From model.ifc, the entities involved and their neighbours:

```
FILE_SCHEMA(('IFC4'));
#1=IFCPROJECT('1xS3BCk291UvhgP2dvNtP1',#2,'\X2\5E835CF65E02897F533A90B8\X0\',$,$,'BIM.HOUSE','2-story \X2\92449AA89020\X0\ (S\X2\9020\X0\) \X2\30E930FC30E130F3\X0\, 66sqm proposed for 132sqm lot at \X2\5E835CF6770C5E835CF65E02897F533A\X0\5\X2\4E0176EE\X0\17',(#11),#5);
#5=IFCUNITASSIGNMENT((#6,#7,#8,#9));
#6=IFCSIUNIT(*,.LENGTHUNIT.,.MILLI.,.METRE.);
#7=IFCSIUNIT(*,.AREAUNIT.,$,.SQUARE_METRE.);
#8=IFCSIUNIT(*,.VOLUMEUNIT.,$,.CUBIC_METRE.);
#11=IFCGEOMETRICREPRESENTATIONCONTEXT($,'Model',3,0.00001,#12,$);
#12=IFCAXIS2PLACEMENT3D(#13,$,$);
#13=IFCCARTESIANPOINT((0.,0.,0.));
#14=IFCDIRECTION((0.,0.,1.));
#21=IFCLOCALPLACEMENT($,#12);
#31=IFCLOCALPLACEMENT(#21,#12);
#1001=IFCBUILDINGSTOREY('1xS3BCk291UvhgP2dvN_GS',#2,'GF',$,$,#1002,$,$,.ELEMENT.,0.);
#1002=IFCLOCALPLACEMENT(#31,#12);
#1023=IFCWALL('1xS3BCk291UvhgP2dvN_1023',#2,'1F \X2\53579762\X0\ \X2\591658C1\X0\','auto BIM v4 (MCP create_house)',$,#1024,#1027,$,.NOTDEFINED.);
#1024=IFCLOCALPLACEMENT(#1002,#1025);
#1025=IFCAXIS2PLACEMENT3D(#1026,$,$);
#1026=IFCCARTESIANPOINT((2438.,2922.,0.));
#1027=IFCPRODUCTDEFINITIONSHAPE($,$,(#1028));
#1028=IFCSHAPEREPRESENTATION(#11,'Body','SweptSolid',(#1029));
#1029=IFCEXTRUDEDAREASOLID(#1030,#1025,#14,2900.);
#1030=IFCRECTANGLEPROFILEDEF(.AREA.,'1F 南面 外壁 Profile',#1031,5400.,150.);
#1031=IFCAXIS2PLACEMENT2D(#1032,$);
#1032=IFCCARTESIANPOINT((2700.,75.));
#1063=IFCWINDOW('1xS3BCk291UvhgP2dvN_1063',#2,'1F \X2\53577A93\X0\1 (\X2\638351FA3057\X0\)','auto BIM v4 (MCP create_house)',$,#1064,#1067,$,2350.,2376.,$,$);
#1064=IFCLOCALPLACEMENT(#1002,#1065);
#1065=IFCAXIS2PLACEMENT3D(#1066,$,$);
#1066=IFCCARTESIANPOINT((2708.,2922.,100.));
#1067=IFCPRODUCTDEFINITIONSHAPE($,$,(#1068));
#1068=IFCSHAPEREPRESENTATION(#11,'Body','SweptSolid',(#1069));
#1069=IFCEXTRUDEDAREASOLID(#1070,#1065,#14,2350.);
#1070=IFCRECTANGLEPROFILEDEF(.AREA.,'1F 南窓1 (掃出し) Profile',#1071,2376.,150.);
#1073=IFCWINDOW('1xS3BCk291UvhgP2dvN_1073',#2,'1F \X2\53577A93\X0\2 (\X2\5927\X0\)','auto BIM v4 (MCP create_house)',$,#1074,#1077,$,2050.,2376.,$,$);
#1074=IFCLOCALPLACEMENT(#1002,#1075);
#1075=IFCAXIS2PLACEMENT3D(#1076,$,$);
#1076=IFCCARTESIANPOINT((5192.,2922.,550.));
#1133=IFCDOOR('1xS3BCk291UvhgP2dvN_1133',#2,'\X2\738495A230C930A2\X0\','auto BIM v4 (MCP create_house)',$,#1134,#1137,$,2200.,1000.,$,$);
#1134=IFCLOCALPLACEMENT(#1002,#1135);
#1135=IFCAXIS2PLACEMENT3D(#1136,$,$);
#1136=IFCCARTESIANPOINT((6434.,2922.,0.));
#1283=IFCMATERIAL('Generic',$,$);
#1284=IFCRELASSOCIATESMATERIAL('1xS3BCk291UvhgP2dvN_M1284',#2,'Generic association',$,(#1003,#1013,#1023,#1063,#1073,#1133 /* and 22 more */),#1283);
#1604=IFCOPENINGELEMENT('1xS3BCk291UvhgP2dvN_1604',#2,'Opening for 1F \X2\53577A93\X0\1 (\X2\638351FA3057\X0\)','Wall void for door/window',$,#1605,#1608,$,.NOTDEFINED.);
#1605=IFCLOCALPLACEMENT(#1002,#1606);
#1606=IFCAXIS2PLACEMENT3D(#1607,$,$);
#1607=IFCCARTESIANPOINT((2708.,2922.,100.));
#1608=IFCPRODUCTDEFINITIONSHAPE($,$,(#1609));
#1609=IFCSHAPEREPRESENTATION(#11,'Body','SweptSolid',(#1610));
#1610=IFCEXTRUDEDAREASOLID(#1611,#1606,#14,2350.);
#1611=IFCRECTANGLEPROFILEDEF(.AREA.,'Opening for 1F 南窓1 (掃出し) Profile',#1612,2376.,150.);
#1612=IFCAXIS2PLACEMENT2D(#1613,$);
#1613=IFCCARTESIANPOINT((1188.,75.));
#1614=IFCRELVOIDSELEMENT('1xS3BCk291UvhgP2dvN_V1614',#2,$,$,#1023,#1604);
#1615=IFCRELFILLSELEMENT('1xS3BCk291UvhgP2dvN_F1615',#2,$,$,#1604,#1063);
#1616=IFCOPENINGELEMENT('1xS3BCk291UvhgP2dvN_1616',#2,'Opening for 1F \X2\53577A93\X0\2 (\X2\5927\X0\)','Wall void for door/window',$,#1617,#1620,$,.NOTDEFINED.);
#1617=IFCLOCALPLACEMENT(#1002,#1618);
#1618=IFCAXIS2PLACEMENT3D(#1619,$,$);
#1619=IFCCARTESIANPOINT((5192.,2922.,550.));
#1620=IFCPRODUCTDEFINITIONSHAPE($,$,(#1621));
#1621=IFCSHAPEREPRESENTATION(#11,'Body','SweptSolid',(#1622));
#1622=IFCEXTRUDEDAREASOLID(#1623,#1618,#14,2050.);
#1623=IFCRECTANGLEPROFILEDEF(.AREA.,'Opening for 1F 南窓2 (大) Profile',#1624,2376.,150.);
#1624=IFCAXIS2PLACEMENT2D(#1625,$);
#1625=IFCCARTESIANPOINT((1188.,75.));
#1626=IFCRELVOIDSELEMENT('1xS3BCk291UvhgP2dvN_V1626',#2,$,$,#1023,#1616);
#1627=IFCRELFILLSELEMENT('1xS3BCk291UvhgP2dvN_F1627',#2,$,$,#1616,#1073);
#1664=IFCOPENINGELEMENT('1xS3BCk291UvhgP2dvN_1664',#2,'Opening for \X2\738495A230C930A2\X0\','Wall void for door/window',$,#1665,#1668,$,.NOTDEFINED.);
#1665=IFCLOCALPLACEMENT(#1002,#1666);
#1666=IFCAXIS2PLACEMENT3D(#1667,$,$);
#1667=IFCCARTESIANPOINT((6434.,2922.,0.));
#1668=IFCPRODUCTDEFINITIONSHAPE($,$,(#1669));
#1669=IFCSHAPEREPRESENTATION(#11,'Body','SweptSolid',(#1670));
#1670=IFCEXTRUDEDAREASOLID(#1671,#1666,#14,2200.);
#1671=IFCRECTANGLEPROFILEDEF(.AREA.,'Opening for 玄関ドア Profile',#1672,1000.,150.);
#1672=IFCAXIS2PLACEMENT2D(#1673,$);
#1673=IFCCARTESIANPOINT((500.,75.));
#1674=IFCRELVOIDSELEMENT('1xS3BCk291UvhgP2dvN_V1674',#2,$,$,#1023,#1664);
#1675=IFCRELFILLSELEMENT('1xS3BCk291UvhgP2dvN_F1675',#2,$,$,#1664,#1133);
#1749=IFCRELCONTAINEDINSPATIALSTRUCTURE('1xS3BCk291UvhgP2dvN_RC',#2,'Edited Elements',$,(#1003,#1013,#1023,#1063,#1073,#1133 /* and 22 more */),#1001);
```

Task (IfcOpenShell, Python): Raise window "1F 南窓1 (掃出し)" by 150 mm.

```python
import numpy as np
import ifcopenshell
import ifcopenshell.api.geometry
import ifcopenshell.util.placement
import ifcopenshell.util.unit

model = ifcopenshell.open("model.ifc")
unit_scale = ifcopenshell.util.unit.calculate_unit_scale(model)

window = model.by_guid("1xS3BCk291UvhgP2dvN_1063")
opening = window.FillsVoids[0].RelatingOpeningElement
dz = 150.0

shift = np.array([0.0, 0.0, dz])
# The window is not placed relative to its opening, so move both.
for product in (opening, window):
    matrix = ifcopenshell.util.placement.get_local_placement(product.ObjectPlacement)
    matrix[:3, 3] += shift
    ifcopenshell.api.geometry.edit_object_placement(model, product=product, matrix=matrix, is_si=False)

print(f"moved by {dz * unit_scale:+.3f} m")

model.write("model-out.ifc")
```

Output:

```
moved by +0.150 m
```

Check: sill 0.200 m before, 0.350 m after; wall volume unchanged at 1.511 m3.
